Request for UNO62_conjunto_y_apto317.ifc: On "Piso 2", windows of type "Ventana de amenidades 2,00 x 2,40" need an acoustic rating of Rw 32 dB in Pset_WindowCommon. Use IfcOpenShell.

First a look at what the model holds.

```python
import ifcopenshell
import ifcopenshell.util.element

model = ifcopenshell.open("UNO62_conjunto_y_apto317.ifc")
print(model.schema)
storey = next(s for s in model.by_type("IfcBuildingStorey") if s.Name == "Piso 2")
windows = [e for e in ifcopenshell.util.element.get_decomposition(storey) if e.is_a("IfcWindow")]
seen = {}
for e in windows:
    element_type = ifcopenshell.util.element.get_type(e)
    key = (element_type.Name if element_type != e and element_type else None, ifcopenshell.util.element.get_pset(e, "Pset_WindowCommon", "AcousticRating"))
    seen[key] = seen.get(key, 0) + 1
for (name, value), count in sorted(seen.items(), key=str):
    print(count, "x", name, "|", value)
```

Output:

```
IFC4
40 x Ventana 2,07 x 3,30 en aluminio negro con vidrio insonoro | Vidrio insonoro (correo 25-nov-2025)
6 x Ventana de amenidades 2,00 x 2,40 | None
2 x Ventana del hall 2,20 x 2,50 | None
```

```python
import ifcopenshell
import ifcopenshell.api.pset
import ifcopenshell.util.element

model = ifcopenshell.open("UNO62_conjunto_y_apto317.ifc")

storey = next(s for s in model.by_type("IfcBuildingStorey") if s.Name == "Piso 2")
windows = [e for e in ifcopenshell.util.element.get_decomposition(storey) if e.is_a("IfcWindow")]

count = 0
for e in windows:
    element_type = ifcopenshell.util.element.get_type(e)
    if element_type in (None, e) or element_type.Name != "Ventana de amenidades 2,00 x 2,40":
        continue
    found = ifcopenshell.util.element.get_pset(e, "Pset_WindowCommon", should_inherit=False)
    if found:
        pset = model.by_id(found["id"])
        if len(ifcopenshell.util.element.get_elements_by_pset(pset)) > 1:
            pset = ifcopenshell.api.pset.unshare_pset(model, products=[e], pset=pset)[0]
    else:
        pset = ifcopenshell.api.pset.add_pset(model, product=e, name="Pset_WindowCommon")
    ifcopenshell.api.pset.edit_pset(model, pset=pset, properties={"AcousticRating": "Rw 32 dB"})
    count += 1

print(count, "windows updated")

model.write("UNO62_conjunto_y_apto317_v2.ifc")
```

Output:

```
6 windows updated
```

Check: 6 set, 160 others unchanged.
